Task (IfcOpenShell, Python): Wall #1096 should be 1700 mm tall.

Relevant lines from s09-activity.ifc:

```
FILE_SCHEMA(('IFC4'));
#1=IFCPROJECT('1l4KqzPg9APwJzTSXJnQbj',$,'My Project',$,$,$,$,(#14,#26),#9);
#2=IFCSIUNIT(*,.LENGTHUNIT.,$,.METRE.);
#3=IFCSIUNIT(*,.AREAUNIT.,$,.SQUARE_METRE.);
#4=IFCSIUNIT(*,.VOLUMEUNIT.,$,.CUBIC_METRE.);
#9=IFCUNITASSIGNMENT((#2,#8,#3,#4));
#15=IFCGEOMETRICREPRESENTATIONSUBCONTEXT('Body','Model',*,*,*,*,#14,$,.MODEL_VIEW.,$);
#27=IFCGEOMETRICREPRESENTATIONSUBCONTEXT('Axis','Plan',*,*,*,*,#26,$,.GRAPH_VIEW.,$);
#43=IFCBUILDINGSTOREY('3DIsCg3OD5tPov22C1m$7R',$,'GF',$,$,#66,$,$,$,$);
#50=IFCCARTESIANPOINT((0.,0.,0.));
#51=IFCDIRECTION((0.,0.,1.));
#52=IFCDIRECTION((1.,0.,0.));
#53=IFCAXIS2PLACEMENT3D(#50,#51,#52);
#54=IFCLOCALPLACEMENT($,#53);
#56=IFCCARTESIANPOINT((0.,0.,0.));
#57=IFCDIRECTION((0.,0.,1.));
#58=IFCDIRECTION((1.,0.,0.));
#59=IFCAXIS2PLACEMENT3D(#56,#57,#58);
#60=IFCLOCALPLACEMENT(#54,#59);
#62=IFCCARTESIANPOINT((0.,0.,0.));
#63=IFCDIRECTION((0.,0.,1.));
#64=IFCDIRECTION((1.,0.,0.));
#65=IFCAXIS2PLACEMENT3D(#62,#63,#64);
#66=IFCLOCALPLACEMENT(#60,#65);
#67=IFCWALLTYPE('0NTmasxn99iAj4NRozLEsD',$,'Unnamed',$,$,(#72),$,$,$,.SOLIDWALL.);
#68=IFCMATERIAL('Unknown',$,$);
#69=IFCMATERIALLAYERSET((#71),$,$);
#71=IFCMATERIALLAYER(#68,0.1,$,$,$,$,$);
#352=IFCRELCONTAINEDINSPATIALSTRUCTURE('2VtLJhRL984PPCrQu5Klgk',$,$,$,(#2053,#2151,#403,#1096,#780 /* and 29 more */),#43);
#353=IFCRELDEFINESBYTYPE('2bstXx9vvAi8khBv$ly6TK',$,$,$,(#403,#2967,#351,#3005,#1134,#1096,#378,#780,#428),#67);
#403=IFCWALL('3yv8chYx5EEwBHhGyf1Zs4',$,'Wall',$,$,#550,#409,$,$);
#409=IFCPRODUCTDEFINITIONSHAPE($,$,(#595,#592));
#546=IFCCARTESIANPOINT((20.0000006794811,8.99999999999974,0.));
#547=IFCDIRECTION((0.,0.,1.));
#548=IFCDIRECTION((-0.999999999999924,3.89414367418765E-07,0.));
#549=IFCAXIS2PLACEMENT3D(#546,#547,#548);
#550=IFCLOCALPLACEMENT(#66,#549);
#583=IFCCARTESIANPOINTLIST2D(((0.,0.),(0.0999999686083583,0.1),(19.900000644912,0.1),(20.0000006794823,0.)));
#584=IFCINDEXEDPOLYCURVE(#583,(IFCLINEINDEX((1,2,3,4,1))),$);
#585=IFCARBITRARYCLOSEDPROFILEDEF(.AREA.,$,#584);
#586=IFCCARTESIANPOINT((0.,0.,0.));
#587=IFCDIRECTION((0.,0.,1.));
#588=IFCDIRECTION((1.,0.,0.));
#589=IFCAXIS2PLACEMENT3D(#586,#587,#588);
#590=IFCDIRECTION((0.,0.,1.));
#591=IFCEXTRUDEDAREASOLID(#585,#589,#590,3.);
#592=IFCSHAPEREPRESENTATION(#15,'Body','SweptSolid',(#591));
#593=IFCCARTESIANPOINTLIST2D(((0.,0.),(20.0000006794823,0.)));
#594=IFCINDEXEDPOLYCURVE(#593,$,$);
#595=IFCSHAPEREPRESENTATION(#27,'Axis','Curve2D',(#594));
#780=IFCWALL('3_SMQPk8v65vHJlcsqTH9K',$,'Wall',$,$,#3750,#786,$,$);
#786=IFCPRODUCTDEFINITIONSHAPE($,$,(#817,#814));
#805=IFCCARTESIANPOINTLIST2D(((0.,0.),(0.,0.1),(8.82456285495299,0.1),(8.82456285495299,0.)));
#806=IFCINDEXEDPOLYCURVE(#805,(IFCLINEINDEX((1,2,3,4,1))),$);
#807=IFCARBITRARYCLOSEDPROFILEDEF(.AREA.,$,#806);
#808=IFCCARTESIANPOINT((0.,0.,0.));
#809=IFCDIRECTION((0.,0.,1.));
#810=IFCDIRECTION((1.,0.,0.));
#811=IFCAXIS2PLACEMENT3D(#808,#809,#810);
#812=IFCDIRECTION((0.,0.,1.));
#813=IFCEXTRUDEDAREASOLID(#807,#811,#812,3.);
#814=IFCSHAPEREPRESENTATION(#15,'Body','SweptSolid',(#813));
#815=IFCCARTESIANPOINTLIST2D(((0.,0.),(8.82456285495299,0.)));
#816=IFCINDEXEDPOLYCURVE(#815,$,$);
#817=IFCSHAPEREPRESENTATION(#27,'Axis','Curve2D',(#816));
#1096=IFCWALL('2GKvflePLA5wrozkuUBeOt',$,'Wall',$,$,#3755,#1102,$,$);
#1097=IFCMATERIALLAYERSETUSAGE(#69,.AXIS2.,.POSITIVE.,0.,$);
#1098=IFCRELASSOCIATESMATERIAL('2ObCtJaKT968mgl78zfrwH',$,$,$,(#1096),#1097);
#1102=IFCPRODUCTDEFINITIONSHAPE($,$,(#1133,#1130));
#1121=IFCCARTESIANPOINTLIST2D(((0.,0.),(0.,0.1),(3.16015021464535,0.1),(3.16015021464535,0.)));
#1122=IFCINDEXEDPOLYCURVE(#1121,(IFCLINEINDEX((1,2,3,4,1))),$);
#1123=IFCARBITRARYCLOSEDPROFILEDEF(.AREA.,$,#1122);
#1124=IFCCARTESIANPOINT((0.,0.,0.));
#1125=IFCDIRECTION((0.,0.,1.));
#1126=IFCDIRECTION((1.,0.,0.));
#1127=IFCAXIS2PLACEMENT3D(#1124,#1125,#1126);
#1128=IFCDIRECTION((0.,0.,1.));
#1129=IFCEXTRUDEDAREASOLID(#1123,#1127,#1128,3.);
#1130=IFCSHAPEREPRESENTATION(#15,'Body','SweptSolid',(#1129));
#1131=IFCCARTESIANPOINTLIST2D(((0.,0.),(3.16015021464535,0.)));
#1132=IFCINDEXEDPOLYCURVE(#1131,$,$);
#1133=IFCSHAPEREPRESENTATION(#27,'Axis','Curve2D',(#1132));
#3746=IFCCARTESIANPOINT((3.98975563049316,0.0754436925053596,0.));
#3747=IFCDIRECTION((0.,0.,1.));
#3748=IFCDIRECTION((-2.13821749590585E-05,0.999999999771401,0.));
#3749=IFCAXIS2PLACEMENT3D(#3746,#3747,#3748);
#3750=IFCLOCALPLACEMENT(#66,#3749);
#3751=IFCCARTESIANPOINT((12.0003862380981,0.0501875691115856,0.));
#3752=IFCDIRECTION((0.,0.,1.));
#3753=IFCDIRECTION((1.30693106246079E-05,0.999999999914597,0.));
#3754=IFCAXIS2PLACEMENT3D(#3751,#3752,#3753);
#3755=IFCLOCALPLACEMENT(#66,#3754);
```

```python
import ifcopenshell
import ifcopenshell.geom
import ifcopenshell.util.representation
import ifcopenshell.util.shape

model = ifcopenshell.open("s09-activity.ifc")
settings = ifcopenshell.geom.settings()


def volume(element):
    """Net volume in cubic metres, openings subtracted."""
    shape = ifcopenshell.geom.create_shape(settings, element)
    return ifcopenshell.util.shape.get_volume(shape.geometry)


wall = model.by_guid("2GKvflePLA5wrozkuUBeOt")
before = volume(wall)

body = ifcopenshell.util.representation.get_representation(wall, "Model", "Body")
solid = body.Items[0]
old_height = solid.Depth
solid.Depth = 1.7
after = volume(wall)

print(f"height {old_height:g} -> {solid.Depth:g}, volume {before:.3f} -> {after:.3f} m3")

model.write("s09-activity_v2.ifc")
```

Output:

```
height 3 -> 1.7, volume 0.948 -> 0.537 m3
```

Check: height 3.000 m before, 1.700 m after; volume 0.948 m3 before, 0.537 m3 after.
